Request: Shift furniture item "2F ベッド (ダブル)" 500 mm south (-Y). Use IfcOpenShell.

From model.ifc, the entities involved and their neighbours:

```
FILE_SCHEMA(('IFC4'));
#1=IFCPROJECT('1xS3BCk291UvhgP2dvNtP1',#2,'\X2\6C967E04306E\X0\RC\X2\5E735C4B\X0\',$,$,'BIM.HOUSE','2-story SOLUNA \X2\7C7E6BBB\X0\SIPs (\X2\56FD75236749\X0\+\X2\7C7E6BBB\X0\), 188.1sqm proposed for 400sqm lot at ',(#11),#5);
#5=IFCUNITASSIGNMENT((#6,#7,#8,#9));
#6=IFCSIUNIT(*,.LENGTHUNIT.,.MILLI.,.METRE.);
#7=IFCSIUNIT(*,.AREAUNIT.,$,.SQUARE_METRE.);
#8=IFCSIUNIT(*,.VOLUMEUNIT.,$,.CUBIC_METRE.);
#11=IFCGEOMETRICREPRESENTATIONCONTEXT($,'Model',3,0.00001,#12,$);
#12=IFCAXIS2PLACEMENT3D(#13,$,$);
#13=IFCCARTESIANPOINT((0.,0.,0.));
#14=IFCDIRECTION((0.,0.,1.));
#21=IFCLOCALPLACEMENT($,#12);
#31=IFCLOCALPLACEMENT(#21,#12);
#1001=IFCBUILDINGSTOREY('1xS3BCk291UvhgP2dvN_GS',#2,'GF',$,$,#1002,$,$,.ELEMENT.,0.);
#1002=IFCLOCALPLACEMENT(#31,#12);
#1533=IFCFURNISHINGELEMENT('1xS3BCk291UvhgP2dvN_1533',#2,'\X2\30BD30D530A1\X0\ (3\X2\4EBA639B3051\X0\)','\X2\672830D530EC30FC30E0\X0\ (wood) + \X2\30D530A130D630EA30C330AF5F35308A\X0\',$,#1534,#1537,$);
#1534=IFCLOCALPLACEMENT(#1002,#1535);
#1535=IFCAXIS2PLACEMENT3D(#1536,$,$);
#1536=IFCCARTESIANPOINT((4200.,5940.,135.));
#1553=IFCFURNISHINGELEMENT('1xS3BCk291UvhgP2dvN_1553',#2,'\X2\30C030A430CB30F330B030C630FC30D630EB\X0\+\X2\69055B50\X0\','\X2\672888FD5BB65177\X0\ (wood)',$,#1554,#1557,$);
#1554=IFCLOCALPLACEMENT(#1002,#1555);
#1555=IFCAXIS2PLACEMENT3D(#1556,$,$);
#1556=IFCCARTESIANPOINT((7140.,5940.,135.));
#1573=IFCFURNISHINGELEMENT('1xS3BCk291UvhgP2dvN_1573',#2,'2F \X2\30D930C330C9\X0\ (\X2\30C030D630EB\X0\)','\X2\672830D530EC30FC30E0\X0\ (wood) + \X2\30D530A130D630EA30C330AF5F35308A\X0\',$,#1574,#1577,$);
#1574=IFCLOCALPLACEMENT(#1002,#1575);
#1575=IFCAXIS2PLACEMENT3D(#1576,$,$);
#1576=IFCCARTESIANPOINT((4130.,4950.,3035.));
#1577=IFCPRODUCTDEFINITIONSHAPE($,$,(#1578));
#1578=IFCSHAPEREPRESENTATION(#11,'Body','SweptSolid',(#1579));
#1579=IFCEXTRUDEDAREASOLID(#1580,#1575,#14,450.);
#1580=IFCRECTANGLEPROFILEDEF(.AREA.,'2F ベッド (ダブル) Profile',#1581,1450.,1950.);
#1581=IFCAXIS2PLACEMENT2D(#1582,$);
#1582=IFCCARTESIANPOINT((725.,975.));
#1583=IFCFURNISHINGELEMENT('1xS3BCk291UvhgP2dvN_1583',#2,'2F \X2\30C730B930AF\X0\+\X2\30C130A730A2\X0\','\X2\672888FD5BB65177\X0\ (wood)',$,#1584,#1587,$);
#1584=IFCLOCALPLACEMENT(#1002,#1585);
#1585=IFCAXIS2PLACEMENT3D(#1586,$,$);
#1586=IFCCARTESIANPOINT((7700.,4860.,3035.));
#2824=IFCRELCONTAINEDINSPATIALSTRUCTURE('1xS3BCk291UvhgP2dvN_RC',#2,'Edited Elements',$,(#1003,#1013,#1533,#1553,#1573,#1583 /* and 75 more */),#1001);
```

```python
import ifcopenshell
import ifcopenshell.api.geometry
import ifcopenshell.util.placement
import ifcopenshell.util.unit

model = ifcopenshell.open("model.ifc")
unit_scale = ifcopenshell.util.unit.calculate_unit_scale(model)

item = model.by_id(1573)
matrix = ifcopenshell.util.placement.get_local_placement(item.ObjectPlacement)
matrix[1, 3] -= 0.5 / unit_scale
ifcopenshell.api.geometry.edit_object_placement(model, product=item, matrix=matrix, is_si=False)

print(ifcopenshell.util.placement.get_local_placement(item.ObjectPlacement).round(3) + 0.0)

model.write("model_rev.ifc")
```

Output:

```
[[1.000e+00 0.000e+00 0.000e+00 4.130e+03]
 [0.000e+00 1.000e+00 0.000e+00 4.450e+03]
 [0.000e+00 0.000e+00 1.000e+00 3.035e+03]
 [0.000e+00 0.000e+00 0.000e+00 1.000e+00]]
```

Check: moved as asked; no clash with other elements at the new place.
